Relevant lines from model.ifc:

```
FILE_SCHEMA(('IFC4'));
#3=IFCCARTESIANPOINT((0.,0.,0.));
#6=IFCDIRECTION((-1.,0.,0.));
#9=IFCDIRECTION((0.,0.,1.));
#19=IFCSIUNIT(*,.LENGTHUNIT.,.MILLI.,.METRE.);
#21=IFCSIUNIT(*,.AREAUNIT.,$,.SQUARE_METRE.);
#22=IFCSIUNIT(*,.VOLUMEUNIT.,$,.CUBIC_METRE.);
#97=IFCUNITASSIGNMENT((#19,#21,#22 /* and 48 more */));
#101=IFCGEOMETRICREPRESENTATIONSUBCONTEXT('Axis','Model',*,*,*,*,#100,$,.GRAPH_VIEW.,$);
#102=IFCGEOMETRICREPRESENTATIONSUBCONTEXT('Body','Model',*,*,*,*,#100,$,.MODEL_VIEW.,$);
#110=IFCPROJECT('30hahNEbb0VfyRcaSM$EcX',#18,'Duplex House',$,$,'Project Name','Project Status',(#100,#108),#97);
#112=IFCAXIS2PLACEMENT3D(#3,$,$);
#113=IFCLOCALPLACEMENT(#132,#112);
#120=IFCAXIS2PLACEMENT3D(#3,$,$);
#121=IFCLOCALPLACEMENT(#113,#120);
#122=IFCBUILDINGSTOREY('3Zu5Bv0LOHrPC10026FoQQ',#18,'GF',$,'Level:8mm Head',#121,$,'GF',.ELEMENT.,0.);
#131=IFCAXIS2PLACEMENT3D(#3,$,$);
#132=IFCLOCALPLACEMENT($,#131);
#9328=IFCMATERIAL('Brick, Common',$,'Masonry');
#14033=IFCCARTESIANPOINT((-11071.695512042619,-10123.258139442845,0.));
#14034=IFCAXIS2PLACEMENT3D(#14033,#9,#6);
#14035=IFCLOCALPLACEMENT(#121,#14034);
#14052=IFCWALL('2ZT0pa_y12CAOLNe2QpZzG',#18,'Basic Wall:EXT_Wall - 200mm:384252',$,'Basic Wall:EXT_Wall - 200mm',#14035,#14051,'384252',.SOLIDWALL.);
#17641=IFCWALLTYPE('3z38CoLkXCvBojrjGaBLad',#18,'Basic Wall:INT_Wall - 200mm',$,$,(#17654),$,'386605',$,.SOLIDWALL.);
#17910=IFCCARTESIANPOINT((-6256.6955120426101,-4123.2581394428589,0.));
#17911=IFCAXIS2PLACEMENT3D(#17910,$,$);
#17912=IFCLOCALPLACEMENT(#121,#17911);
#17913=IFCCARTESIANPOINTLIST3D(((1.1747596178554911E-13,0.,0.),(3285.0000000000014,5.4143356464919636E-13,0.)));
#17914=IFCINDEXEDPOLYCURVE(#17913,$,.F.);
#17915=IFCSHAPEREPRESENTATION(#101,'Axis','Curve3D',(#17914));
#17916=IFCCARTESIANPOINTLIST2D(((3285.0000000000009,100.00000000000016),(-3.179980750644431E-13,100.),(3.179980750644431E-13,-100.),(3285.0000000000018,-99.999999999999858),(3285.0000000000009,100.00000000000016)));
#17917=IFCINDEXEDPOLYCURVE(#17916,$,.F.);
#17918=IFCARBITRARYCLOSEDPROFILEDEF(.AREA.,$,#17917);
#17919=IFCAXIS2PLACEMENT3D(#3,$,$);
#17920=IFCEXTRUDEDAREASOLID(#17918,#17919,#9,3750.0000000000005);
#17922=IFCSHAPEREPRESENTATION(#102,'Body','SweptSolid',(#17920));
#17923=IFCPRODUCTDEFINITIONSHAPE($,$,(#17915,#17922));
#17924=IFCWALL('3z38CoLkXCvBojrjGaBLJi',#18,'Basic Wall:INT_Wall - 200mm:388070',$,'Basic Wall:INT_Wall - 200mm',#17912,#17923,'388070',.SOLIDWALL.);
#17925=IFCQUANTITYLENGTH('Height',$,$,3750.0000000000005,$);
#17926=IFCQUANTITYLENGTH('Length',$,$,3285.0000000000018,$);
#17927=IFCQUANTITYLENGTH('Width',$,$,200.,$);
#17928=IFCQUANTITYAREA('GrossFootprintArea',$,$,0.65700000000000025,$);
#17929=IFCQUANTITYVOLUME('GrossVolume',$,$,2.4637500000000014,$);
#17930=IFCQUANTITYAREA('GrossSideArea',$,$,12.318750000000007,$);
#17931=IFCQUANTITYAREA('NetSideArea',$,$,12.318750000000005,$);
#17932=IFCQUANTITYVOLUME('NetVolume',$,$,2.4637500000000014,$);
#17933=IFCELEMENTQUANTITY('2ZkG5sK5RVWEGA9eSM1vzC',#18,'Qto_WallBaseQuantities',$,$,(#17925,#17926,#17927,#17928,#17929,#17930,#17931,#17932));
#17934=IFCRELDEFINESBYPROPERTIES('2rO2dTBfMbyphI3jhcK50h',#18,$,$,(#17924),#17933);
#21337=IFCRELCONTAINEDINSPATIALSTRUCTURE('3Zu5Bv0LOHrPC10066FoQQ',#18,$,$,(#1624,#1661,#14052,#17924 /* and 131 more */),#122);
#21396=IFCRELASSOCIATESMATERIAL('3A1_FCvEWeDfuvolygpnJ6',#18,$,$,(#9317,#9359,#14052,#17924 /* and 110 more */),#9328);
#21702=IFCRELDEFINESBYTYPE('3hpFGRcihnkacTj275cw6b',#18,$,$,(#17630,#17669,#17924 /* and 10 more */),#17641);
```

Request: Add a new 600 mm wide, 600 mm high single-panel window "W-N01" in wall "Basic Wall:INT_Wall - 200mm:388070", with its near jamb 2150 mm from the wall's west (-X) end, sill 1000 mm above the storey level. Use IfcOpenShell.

```python
import numpy as np
import ifcopenshell
import ifcopenshell.api.feature
import ifcopenshell.api.geometry
import ifcopenshell.api.pset
import ifcopenshell.api.root
import ifcopenshell.api.spatial
import ifcopenshell.geom
import ifcopenshell.util.element
import ifcopenshell.util.placement
import ifcopenshell.util.representation
import ifcopenshell.util.shape
import ifcopenshell.util.unit

model = ifcopenshell.open("model.ifc")
unit_scale = ifcopenshell.util.unit.calculate_unit_scale(model)
area_scale = ifcopenshell.util.unit.calculate_unit_scale(model, "AREAUNIT")
volume_scale = ifcopenshell.util.unit.calculate_unit_scale(model, "VOLUMEUNIT")
settings = ifcopenshell.geom.settings()


def volume(element):
    """Net volume in cubic metres, openings subtracted."""
    shape = ifcopenshell.geom.create_shape(settings, element)
    return ifcopenshell.util.shape.get_volume(shape.geometry)


wall = model.by_guid("3z38CoLkXCvBojrjGaBLJi")
storey = ifcopenshell.util.element.get_container(wall, ifc_class="IfcBuildingStorey")
context = ifcopenshell.util.representation.get_context(model, "Model", "Body", "MODEL_VIEW")
before = volume(wall)

width, height, from_end, sill = 0.6, 0.6, 2.15, 1  # metres

# The wall runs along its own X axis, and the end named is its -X end.
wall_shape = ifcopenshell.geom.create_shape(settings, wall)
x, y, z = ifcopenshell.util.shape.get_vertices(wall_shape.geometry).T
start = x.min() + from_end
face, thickness = float(y.min()), float(y.max() - y.min())
wall_matrix = ifcopenshell.util.placement.get_local_placement(wall.ObjectPlacement)
level = ifcopenshell.util.placement.get_local_placement(storey.ObjectPlacement)[2, 3]


def in_wall(x, y):
    """Placement at x, y metres in the wall's axes, at sill height."""
    matrix = wall_matrix.copy()
    matrix[:, 3] = wall_matrix @ np.array([x / unit_scale, y / unit_scale, 0.0, 1.0])
    matrix[2, 3] = level + sill / unit_scale
    return matrix


# Opening: a box that overshoots both wall faces by 50 mm.
opening = ifcopenshell.api.root.create_entity(model, ifc_class="IfcOpeningElement", predefined_type="OPENING")
box = ifcopenshell.api.geometry.add_wall_representation(
    model, context=context, length=width, height=height, thickness=thickness + 0.1
)
ifcopenshell.api.geometry.assign_representation(model, product=opening, representation=box)
ifcopenshell.api.geometry.edit_object_placement(model, product=opening, matrix=in_wall(start, face - 0.05), is_si=False)
ifcopenshell.api.feature.add_feature(model, feature=opening, element=wall)

window = ifcopenshell.api.root.create_entity(model, ifc_class="IfcWindow", name="W-N01", predefined_type="WINDOW")
window.OverallWidth, window.OverallHeight = width / unit_scale, height / unit_scale
window.PartitioningType = "SINGLE_PANEL"
body = ifcopenshell.api.geometry.add_window_representation(
    model,
    context=context,
    overall_width=window.OverallWidth,
    overall_height=window.OverallHeight,
    partition_type="SINGLE_PANEL",
)
ifcopenshell.api.geometry.assign_representation(model, product=window, representation=body)
ifcopenshell.api.spatial.assign_container(model, products=[window], relating_structure=storey)
ifcopenshell.api.feature.add_filling(model, opening=opening, element=window)

# Centre the window in the wall's thickness.
ifcopenshell.api.geometry.edit_object_placement(model, product=window, matrix=in_wall(start, face), is_si=False)
window_shape = ifcopenshell.geom.create_shape(settings, window)
depth = ifcopenshell.util.shape.get_vertices(window_shape.geometry)[:, 1]
offset = face + thickness / 2 - (depth.min() + depth.max()) / 2
ifcopenshell.api.geometry.edit_object_placement(model, product=window, matrix=in_wall(start, offset), is_si=False)

after = volume(wall)

# Update the wall's stored quantities.
qto = model.by_id(ifcopenshell.util.element.get_pset(wall, "Qto_WallBaseQuantities", should_inherit=False)["id"])
ifcopenshell.api.pset.edit_qto(model, qto=qto, properties={
    "NetSideArea": after / thickness / area_scale,
    "NetVolume": after / volume_scale,
})

print(f"wall volume {before:.3f} -> {after:.3f} m3")

model.write("model_v2.ifc")
```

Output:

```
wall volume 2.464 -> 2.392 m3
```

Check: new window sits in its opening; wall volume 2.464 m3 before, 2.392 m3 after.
